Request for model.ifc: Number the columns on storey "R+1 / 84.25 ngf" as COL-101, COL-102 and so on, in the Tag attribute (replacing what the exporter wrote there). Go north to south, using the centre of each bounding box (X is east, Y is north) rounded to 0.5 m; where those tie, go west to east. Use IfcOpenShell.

First a look at what the model holds.

```python
import ifcopenshell
import ifcopenshell.util.element
import ifcopenshell.util.placement

model = ifcopenshell.open("model.ifc")
print(model.schema)
storey = next(s for s in model.by_type("IfcBuildingStorey") if s.Name == "R+1 / 84.25 ngf")
columns = [e for e in ifcopenshell.util.element.get_decomposition(storey) if e.is_a("IfcColumn")]
for e in sorted(columns, key=lambda e: e.id()):
    origin = ifcopenshell.util.placement.get_local_placement(e.ObjectPlacement)[:3, 3]
    print(e.id(), e.Tag, e.Name, origin.round(2) + 0.0, sep=" | ")
```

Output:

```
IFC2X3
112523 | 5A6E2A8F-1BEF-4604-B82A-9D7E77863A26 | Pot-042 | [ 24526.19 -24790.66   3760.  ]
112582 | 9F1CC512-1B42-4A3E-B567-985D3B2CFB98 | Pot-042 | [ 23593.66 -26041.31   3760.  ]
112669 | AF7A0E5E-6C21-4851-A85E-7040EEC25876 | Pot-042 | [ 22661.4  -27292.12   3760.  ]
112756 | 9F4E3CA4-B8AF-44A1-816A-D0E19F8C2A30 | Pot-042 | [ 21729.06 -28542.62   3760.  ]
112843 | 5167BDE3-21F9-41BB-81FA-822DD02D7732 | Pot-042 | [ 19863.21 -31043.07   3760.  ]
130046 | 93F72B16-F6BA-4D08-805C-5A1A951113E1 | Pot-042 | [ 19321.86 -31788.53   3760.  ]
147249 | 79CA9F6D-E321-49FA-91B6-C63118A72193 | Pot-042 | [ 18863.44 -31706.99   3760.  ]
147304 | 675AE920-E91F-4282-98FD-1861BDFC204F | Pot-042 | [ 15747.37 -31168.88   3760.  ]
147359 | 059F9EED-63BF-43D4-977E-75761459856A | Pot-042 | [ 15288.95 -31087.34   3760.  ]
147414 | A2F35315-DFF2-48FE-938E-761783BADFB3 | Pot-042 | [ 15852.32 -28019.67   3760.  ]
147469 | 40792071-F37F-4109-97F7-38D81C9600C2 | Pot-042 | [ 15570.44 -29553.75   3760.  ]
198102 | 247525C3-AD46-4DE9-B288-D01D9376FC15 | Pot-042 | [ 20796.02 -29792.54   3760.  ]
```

```python
import ifcopenshell
import ifcopenshell.geom
import ifcopenshell.util.element
import ifcopenshell.util.shape

model = ifcopenshell.open("model.ifc")
settings = ifcopenshell.geom.settings()
settings.set("use-world-coords", True)


def centre(element):
    shape = ifcopenshell.geom.create_shape(settings, element)
    return ifcopenshell.util.shape.get_bbox_centroid(shape.geometry)


storey = next(s for s in model.by_type("IfcBuildingStorey") if s.Name == "R+1 / 84.25 ngf")
columns = [e for e in ifcopenshell.util.element.get_decomposition(storey) if e.is_a("IfcColumn")]

# Insertion points can sit at a corner or the storey origin, so sort by the geometry (in metres).
centres = {e: centre(e) for e in columns}
columns.sort(key=lambda e: (-round(centres[e][1] / 0.5), centres[e][0]))

for i, e in enumerate(columns, start=1):
    number = f"COL-1{i:02d}"
    e.Tag = number
    print(e.id(), number)

model.write("model_updated.ifc")
```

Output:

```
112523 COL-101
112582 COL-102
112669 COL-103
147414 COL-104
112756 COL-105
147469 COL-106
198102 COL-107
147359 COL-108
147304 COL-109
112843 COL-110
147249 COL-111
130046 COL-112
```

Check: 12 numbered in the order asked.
